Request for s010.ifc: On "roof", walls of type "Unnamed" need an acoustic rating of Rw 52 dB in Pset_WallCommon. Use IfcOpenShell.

First a look at what the model holds.

```python
import ifcopenshell
import ifcopenshell.util.element

model = ifcopenshell.open("s010.ifc")
print(model.schema)
storey = next(s for s in model.by_type("IfcBuildingStorey") if s.Name == "roof")
walls = [e for e in ifcopenshell.util.element.get_decomposition(storey) if e.is_a("IfcWall")]
seen = {}
for e in walls:
    element_type = ifcopenshell.util.element.get_type(e)
    key = (element_type.Name if element_type != e and element_type else None, ifcopenshell.util.element.get_pset(e, "Pset_WallCommon", "AcousticRating"))
    seen[key] = seen.get(key, 0) + 1
for (name, value), count in sorted(seen.items(), key=str):
    print(count, "x", name, "|", value)
```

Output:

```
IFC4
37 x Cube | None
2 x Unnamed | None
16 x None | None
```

```python
import ifcopenshell
import ifcopenshell.api.pset
import ifcopenshell.util.element

model = ifcopenshell.open("s010.ifc")

storey = next(s for s in model.by_type("IfcBuildingStorey") if s.Name == "roof")
walls = [e for e in ifcopenshell.util.element.get_decomposition(storey) if e.is_a("IfcWall")]

count = 0
for e in walls:
    element_type = ifcopenshell.util.element.get_type(e)
    if element_type in (None, e) or element_type.Name != "Unnamed":
        continue
    # add_pset returns the element's existing set when there is one.
    pset = ifcopenshell.api.pset.add_pset(model, product=e, name="Pset_WallCommon")
    ifcopenshell.api.pset.edit_pset(model, pset=pset, properties={"AcousticRating": "Rw 52 dB"})
    count += 1

print(count, "walls updated")

model.write("s010_updated.ifc")
```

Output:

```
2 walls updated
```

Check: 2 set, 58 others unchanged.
